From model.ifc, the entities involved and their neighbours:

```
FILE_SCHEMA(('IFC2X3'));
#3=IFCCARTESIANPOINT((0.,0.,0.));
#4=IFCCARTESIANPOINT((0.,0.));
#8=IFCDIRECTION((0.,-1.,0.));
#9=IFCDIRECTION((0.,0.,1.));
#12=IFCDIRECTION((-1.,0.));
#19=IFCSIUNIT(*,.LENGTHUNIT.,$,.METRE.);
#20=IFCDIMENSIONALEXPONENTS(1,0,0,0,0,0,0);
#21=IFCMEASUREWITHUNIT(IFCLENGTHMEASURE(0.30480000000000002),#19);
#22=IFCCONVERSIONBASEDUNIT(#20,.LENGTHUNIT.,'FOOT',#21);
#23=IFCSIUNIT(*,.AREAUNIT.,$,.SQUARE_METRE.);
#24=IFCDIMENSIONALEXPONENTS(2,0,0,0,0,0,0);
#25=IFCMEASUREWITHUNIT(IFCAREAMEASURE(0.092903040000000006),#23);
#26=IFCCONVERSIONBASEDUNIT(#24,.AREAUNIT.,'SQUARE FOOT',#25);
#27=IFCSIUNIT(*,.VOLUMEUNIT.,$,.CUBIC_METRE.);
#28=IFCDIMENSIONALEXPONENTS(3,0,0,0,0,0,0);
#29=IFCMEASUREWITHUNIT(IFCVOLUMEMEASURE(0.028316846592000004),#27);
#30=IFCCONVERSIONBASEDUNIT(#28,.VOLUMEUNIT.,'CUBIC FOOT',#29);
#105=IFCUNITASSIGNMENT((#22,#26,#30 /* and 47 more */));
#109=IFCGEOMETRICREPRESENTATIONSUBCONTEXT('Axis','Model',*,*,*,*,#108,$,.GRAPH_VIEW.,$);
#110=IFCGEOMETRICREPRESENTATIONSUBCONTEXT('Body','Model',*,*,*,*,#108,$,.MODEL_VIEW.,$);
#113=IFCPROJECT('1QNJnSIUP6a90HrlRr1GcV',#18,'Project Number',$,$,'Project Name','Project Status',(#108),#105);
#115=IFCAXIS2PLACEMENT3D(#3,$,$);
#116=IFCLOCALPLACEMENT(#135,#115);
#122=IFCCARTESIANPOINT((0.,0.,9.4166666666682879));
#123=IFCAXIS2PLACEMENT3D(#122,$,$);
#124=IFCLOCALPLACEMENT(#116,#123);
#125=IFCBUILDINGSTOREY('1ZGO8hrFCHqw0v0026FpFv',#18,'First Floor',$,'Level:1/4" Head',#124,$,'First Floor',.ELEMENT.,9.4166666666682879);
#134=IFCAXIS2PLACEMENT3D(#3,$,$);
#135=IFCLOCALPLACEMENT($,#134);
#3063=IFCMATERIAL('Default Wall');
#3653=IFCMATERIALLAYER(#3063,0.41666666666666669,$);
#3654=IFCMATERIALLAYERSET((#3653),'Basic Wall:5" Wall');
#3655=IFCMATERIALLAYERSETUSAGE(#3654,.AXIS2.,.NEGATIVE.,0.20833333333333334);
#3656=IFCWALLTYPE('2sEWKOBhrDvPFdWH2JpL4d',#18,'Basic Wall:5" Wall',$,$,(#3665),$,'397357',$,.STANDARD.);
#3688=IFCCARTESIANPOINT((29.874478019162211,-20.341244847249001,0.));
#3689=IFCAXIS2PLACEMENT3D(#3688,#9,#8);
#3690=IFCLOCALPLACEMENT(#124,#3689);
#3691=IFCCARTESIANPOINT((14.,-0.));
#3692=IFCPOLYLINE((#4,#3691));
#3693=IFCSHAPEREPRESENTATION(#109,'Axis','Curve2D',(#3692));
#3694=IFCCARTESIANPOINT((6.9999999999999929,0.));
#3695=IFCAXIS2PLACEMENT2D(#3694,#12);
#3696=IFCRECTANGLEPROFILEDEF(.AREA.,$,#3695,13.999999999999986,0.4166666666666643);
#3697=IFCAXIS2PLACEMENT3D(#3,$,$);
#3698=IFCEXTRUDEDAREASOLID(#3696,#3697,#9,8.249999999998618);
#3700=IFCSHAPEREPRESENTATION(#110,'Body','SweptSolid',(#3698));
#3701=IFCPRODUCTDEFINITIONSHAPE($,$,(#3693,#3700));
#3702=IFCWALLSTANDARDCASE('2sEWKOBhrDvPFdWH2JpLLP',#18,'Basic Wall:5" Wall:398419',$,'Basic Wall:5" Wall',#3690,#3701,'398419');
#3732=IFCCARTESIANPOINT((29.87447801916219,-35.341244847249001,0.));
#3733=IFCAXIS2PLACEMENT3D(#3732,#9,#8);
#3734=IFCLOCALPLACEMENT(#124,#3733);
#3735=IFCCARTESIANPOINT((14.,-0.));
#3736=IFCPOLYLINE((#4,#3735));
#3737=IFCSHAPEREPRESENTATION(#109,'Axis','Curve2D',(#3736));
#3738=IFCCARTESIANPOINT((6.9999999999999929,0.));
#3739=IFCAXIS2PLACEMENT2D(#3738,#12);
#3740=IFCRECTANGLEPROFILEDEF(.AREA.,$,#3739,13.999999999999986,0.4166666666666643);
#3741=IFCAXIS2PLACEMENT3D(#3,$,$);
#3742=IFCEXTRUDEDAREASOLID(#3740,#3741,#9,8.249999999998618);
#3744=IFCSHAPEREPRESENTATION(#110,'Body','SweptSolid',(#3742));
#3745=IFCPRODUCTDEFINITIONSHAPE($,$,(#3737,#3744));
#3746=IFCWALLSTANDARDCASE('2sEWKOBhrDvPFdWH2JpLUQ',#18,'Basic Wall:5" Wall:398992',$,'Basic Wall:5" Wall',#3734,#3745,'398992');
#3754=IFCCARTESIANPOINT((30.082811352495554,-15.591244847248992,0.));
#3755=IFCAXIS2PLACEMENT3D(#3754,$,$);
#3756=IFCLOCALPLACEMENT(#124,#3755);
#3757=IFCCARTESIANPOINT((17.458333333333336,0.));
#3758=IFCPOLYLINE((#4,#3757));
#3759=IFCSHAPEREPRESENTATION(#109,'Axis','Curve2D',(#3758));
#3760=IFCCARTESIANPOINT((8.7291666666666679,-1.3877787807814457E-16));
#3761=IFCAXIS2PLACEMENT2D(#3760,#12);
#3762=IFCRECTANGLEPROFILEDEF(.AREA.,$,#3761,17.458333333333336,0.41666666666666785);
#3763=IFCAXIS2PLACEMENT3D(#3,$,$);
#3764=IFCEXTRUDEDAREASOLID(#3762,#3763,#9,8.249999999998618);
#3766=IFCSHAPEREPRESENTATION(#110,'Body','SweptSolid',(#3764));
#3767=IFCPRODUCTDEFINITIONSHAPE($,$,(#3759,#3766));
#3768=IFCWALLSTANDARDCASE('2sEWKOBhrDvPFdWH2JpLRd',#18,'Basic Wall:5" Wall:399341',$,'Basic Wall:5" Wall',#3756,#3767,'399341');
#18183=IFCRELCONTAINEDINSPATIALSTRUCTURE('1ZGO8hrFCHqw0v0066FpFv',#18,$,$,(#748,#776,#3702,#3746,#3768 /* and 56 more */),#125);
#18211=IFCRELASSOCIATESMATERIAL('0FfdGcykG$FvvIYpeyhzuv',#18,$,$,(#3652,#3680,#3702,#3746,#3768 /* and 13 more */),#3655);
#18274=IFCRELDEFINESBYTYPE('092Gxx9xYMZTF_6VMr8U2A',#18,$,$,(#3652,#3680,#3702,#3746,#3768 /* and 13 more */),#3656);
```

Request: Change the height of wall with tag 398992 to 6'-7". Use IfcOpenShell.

```python
import ifcopenshell
import ifcopenshell.geom
import ifcopenshell.util.representation
import ifcopenshell.util.shape
import ifcopenshell.util.unit

model = ifcopenshell.open("model.ifc")
unit_scale = ifcopenshell.util.unit.calculate_unit_scale(model)
settings = ifcopenshell.geom.settings()


def volume(element):
    """Net volume in cubic metres, openings subtracted."""
    shape = ifcopenshell.geom.create_shape(settings, element)
    return ifcopenshell.util.shape.get_volume(shape.geometry)


wall = model.by_guid("2sEWKOBhrDvPFdWH2JpLUQ")
before = volume(wall)

body = ifcopenshell.util.representation.get_representation(wall, "Model", "Body")
solid = body.Items[0]
old_height = solid.Depth
solid.Depth = 79 * 0.0254 / unit_scale
after = volume(wall)

print(f"height {old_height:g} -> {solid.Depth:g}, volume {before:.3f} -> {after:.3f} m3")

model.write("model-out.ifc")
```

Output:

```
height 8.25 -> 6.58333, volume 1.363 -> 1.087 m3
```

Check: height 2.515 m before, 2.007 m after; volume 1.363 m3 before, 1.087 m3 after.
